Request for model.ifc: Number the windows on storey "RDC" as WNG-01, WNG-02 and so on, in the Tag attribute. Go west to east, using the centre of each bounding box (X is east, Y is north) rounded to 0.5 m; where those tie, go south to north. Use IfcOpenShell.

First a look at what the model holds.

```python
import ifcopenshell
import ifcopenshell.util.element
import ifcopenshell.util.placement

model = ifcopenshell.open("model.ifc")
print(model.schema)
storey = next(s for s in model.by_type("IfcBuildingStorey") if s.Name == "RDC")
windows = [e for e in ifcopenshell.util.element.get_decomposition(storey) if e.is_a("IfcWindow")]
for e in sorted(windows, key=lambda e: e.id()):
    origin = ifcopenshell.util.placement.get_local_placement(e.ObjectPlacement)[:3, 3]
    print(e.id(), e.Tag, e.Name, origin.round(2) + 0.0, sep=" | ")
```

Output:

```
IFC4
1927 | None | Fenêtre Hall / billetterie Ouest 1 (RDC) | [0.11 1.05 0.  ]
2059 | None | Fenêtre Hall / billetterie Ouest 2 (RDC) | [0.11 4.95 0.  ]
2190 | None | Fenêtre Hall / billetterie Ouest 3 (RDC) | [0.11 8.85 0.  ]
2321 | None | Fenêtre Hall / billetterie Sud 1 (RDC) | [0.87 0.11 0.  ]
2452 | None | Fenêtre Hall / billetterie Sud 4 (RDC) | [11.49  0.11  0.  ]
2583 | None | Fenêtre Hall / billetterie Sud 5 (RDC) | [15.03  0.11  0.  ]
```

```python
import ifcopenshell
import ifcopenshell.geom
import ifcopenshell.util.element
import ifcopenshell.util.shape

model = ifcopenshell.open("model.ifc")
settings = ifcopenshell.geom.settings()
settings.set("use-world-coords", True)


def centre(element):
    shape = ifcopenshell.geom.create_shape(settings, element)
    return ifcopenshell.util.shape.get_bbox_centroid(shape.geometry)


storey = next(s for s in model.by_type("IfcBuildingStorey") if s.Name == "RDC")
windows = [e for e in ifcopenshell.util.element.get_decomposition(storey) if e.is_a("IfcWindow")]

# Insertion points can sit at a corner or the storey origin, so sort by the geometry (in metres).
centres = {e: centre(e) for e in windows}
windows.sort(key=lambda e: (round(centres[e][0] / 0.5), centres[e][1]))

for i, e in enumerate(windows, start=1):
    number = f"WNG-{i:02d}"
    e.Tag = number
    print(e.id(), number)

model.write("model-out.ifc")
```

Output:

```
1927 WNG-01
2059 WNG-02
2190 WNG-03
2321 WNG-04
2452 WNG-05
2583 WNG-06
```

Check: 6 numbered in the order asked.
